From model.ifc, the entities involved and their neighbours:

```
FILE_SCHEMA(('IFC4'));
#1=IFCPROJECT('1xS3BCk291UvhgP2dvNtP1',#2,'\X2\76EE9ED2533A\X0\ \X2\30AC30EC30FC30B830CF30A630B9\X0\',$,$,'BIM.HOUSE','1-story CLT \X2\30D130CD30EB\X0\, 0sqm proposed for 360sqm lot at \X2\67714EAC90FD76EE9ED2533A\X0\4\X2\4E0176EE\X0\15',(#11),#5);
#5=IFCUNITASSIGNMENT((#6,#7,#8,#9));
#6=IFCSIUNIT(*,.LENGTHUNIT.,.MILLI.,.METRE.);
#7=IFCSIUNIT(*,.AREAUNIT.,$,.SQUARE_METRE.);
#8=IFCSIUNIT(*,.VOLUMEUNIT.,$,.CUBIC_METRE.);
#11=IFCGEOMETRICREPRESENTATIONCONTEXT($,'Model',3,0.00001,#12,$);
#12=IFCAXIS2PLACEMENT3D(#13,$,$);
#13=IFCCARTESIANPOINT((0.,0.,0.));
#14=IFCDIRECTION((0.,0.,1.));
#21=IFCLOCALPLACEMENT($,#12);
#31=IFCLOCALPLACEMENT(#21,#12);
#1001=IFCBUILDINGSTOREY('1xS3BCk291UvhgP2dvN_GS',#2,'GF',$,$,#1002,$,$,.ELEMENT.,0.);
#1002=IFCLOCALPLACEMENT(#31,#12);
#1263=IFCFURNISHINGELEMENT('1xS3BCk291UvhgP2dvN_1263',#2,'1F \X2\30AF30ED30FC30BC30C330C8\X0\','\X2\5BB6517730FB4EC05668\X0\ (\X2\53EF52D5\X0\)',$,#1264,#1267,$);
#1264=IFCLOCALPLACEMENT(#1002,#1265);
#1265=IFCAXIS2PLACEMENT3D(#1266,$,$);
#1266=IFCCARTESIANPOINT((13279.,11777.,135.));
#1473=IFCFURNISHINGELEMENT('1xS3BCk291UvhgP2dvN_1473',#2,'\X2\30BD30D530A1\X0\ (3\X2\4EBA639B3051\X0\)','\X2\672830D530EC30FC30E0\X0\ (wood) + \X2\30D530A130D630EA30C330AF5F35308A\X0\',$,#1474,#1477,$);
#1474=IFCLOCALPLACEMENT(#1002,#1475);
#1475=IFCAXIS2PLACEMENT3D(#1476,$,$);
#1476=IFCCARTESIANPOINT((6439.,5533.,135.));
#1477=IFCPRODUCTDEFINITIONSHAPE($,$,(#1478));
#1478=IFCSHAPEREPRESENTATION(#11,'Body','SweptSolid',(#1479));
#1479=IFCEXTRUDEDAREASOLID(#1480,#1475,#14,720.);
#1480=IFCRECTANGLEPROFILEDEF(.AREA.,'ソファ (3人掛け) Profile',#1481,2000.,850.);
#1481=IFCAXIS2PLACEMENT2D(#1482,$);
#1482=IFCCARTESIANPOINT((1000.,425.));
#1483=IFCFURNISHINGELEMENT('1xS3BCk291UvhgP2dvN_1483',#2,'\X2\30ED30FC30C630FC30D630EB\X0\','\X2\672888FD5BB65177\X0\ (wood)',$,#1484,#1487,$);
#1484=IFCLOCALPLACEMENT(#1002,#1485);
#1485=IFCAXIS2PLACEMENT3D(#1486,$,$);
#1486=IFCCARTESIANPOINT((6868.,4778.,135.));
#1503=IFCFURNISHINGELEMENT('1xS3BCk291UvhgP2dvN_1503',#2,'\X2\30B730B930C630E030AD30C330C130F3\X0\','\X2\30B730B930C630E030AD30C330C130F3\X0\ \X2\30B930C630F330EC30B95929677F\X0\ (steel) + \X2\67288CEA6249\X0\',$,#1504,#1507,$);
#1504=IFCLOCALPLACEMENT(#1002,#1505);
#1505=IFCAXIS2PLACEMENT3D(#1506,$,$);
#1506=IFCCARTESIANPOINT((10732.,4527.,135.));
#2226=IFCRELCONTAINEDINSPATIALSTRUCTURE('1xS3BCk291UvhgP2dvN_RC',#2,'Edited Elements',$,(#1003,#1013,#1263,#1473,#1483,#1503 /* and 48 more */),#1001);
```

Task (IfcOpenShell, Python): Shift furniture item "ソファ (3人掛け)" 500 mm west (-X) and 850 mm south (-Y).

```python
import ifcopenshell
import ifcopenshell.api.geometry
import ifcopenshell.util.placement
import ifcopenshell.util.unit

model = ifcopenshell.open("model.ifc")
unit_scale = ifcopenshell.util.unit.calculate_unit_scale(model)

item = model.by_id(1473)
matrix = ifcopenshell.util.placement.get_local_placement(item.ObjectPlacement)
matrix[0, 3] -= 0.5 / unit_scale
matrix[1, 3] -= 0.85 / unit_scale
ifcopenshell.api.geometry.edit_object_placement(model, product=item, matrix=matrix, is_si=False)

print(ifcopenshell.util.placement.get_local_placement(item.ObjectPlacement).round(3) + 0.0)

model.write("model_v2.ifc")
```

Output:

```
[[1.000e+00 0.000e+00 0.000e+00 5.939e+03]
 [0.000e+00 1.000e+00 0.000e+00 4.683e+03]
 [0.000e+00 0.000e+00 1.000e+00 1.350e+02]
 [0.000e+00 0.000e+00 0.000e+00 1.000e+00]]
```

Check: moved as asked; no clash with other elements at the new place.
